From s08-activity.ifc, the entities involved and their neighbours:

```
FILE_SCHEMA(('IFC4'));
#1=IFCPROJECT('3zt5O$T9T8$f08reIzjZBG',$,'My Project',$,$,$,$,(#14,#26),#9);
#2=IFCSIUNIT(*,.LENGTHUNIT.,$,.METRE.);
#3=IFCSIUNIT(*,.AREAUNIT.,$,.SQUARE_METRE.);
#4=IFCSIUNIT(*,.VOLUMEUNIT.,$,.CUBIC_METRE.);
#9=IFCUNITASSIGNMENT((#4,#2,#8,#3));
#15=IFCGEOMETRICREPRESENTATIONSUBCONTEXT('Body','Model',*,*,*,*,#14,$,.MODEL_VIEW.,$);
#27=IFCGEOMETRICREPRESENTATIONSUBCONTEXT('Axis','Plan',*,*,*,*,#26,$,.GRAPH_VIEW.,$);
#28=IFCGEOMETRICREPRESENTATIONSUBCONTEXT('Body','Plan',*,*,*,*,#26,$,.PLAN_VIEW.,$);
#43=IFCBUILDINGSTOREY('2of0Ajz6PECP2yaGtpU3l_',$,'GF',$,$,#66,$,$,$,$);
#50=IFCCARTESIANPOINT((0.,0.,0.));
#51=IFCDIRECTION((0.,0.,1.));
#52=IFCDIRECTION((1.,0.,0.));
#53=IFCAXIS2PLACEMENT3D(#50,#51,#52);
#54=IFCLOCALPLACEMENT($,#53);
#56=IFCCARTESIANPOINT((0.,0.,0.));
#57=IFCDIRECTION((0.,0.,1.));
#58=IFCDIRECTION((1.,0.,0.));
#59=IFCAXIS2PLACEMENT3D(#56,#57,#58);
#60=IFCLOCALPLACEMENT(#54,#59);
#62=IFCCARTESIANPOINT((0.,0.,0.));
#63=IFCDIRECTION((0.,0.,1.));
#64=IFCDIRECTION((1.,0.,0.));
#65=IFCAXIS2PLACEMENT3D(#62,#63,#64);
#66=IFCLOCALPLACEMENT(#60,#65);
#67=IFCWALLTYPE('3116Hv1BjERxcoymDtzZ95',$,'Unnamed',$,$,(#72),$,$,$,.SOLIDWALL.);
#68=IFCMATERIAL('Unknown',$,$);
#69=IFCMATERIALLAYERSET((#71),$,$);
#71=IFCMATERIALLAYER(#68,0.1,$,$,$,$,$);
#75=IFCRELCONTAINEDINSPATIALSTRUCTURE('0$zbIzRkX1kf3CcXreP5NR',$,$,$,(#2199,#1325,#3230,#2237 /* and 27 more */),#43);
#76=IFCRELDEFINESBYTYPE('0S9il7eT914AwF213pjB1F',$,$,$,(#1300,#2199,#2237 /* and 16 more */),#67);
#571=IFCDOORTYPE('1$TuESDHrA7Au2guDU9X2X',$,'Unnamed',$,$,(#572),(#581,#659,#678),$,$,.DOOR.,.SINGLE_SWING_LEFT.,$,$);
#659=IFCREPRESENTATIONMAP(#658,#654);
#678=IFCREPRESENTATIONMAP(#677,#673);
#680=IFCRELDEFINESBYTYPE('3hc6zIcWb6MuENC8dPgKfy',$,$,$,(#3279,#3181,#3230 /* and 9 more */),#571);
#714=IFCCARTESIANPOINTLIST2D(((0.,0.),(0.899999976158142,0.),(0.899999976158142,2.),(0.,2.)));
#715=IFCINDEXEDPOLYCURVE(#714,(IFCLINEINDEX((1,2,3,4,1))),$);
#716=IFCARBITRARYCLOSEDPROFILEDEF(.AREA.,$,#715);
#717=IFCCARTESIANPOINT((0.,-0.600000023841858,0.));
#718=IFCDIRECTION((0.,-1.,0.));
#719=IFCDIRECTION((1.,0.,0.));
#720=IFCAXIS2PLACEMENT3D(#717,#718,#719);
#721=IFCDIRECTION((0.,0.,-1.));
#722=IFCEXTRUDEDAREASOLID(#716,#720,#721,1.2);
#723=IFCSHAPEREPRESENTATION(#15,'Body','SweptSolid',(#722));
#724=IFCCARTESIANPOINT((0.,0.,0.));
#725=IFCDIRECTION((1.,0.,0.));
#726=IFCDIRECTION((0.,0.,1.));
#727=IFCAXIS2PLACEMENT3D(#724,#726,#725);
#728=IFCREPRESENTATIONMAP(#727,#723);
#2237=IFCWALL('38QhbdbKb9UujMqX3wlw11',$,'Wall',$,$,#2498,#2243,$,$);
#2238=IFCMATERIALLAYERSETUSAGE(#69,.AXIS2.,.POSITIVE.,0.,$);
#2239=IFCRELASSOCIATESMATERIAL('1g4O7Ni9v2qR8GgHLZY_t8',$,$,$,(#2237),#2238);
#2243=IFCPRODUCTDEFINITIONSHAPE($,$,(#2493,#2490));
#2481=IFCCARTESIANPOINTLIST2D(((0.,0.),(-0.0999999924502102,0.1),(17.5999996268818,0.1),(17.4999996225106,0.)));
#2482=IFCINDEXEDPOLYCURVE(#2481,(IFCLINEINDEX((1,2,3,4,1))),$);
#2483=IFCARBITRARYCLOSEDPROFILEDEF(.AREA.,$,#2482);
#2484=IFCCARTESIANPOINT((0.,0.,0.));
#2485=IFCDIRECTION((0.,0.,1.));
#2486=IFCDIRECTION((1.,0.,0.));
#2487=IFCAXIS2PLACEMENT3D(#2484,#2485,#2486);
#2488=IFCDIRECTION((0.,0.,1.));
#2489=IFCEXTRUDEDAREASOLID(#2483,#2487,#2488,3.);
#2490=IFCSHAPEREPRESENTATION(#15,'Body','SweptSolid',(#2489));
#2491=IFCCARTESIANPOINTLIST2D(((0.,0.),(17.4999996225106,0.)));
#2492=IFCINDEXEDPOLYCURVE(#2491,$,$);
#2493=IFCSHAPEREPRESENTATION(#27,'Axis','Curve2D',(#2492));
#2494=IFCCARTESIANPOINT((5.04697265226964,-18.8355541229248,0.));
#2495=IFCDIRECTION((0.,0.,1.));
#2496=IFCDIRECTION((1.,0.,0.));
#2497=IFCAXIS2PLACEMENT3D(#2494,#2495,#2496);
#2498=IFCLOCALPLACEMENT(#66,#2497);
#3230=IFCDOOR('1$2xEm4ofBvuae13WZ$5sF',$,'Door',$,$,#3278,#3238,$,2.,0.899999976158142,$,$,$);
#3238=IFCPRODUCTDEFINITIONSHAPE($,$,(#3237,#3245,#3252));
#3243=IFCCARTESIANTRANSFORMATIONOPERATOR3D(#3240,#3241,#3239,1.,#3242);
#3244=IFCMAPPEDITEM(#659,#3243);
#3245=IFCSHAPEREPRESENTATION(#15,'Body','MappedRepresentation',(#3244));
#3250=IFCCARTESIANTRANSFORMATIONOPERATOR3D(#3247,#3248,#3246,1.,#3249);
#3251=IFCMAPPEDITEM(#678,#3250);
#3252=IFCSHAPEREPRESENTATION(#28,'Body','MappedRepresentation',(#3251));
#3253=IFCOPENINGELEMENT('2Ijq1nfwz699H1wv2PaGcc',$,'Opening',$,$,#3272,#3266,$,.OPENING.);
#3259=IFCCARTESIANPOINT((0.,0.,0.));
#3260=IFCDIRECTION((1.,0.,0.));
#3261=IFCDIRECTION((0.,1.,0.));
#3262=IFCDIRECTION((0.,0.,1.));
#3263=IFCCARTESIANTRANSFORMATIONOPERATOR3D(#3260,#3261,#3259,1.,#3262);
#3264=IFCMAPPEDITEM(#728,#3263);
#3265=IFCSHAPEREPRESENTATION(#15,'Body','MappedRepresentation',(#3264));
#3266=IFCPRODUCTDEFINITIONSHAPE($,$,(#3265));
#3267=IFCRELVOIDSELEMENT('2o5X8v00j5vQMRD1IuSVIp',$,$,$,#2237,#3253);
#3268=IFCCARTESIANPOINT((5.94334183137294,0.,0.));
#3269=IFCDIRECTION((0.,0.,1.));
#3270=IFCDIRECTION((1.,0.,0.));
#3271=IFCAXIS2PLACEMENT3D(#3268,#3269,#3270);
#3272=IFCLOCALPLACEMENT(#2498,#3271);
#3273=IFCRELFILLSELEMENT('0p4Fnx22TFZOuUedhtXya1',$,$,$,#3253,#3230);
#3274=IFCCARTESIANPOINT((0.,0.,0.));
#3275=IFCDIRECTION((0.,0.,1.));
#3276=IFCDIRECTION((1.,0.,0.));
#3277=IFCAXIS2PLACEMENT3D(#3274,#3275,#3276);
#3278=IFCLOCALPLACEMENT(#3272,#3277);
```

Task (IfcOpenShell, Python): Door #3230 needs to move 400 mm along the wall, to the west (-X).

```python
import ifcopenshell
import ifcopenshell.api.geometry
import ifcopenshell.util.placement
import ifcopenshell.util.unit

model = ifcopenshell.open("s08-activity.ifc")
unit_scale = ifcopenshell.util.unit.calculate_unit_scale(model)

door = model.by_guid("1$2xEm4ofBvuae13WZ$5sF")
opening = door.FillsVoids[0].RelatingOpeningElement
wall = opening.VoidsElements[0].RelatingBuildingElement

wall_matrix = ifcopenshell.util.placement.get_local_placement(wall.ObjectPlacement)
shift = wall_matrix[:3, 0] * -0.4 / unit_scale
before = ifcopenshell.util.placement.get_local_placement(door.ObjectPlacement)[:3, 3].copy()

# The door is placed relative to its opening, so it follows when the opening moves.
matrix = ifcopenshell.util.placement.get_local_placement(opening.ObjectPlacement)
matrix[:3, 3] += shift
ifcopenshell.api.geometry.edit_object_placement(
    model, product=opening, matrix=matrix, is_si=False, should_transform_children=True
)

after = ifcopenshell.util.placement.get_local_placement(door.ObjectPlacement)[:3, 3]
print("door moved by", (after - before).round(3) + 0.0)

model.write("s08-activity_edited.ifc")
```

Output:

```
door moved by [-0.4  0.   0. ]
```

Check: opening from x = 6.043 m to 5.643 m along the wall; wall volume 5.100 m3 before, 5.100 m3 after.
